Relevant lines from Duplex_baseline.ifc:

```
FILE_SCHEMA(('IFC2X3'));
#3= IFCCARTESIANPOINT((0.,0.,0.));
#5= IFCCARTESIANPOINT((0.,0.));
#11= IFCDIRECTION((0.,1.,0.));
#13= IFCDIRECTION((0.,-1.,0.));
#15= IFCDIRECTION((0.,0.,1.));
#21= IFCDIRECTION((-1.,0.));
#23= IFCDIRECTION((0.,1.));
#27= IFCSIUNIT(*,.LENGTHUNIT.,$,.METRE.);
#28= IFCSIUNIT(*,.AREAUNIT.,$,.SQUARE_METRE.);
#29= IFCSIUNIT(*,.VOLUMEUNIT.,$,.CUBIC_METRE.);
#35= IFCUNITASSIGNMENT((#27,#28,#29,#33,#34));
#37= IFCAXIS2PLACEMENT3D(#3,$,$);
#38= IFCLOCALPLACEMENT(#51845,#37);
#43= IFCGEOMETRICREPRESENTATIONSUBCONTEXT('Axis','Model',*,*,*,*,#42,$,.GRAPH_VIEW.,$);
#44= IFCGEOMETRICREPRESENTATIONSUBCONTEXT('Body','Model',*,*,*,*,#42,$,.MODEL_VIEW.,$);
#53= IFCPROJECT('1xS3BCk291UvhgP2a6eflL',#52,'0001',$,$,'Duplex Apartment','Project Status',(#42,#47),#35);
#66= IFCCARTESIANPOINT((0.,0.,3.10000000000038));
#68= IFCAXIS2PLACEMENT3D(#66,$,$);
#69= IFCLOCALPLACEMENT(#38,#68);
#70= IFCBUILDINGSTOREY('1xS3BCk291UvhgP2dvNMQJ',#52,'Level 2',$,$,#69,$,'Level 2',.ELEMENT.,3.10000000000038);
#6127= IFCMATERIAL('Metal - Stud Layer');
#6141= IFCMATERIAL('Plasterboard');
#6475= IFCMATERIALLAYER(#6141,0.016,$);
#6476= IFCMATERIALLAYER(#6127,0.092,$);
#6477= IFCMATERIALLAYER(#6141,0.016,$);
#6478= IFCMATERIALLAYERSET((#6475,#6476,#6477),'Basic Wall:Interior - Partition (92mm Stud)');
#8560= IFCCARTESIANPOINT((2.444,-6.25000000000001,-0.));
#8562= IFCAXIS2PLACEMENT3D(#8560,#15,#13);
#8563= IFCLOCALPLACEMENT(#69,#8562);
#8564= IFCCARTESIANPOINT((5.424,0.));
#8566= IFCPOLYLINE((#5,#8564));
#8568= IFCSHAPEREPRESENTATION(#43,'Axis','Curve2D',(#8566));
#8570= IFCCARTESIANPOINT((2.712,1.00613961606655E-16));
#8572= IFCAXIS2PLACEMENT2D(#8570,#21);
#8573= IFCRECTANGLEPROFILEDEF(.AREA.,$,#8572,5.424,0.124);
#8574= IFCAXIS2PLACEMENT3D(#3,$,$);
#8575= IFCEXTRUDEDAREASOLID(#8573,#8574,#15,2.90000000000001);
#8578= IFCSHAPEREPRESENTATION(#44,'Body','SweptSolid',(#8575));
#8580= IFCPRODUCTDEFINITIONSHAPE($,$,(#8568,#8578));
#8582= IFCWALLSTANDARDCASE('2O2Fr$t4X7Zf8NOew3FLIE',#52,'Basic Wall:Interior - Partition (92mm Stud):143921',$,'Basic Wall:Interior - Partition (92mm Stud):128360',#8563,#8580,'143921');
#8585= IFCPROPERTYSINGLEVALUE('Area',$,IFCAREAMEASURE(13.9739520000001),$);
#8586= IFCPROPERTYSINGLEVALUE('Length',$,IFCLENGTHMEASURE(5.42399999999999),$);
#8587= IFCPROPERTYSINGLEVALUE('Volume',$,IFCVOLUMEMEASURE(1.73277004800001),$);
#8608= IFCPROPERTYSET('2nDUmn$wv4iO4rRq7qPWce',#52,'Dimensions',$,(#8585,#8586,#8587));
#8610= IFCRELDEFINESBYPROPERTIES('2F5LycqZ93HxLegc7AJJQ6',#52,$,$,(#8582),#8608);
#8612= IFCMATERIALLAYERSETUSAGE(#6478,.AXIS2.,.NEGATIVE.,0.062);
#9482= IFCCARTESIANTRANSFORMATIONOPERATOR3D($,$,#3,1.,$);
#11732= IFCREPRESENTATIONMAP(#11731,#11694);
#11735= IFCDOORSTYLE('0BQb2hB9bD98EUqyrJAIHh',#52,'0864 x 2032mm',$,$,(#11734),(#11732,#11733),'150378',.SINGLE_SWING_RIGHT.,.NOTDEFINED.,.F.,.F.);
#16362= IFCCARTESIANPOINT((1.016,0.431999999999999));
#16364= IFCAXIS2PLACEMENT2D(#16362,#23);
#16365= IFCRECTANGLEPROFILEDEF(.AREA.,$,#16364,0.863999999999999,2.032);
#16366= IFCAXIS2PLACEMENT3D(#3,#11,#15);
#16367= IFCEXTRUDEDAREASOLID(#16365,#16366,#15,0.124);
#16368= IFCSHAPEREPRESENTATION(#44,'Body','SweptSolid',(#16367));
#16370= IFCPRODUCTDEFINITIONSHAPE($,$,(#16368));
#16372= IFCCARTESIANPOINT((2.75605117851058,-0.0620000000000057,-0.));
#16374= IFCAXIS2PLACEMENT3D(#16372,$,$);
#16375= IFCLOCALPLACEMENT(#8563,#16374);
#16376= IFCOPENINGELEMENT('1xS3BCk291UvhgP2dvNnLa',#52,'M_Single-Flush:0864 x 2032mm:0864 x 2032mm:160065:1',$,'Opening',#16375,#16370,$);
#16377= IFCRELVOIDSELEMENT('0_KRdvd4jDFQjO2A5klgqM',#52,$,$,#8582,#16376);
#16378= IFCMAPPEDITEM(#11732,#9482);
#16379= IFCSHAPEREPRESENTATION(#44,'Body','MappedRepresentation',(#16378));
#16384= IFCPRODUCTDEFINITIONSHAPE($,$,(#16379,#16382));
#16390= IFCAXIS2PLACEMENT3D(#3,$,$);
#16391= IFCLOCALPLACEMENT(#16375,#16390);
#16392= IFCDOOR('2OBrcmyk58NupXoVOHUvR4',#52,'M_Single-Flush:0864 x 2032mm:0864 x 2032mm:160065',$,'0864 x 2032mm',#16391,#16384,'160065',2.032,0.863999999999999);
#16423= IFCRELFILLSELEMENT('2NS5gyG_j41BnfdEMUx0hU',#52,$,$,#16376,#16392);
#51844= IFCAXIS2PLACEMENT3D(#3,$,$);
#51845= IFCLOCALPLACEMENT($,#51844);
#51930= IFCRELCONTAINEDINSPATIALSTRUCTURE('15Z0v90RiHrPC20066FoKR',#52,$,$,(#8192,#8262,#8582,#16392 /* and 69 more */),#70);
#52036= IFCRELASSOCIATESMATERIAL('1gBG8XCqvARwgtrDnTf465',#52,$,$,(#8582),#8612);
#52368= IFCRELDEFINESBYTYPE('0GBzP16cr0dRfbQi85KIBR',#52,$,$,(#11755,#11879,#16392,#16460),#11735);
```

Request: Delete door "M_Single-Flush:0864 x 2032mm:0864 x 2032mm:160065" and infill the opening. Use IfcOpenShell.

```python
import ifcopenshell
import ifcopenshell.api.feature
import ifcopenshell.api.pset
import ifcopenshell.api.root
import ifcopenshell.geom
import ifcopenshell.util.element
import ifcopenshell.util.shape
import ifcopenshell.util.unit

model = ifcopenshell.open("Duplex_baseline.ifc")
area_scale = ifcopenshell.util.unit.calculate_unit_scale(model, "AREAUNIT")
volume_scale = ifcopenshell.util.unit.calculate_unit_scale(model, "VOLUMEUNIT")
settings = ifcopenshell.geom.settings()


def volume(element):
    """Net volume in cubic metres, openings subtracted."""
    shape = ifcopenshell.geom.create_shape(settings, element)
    return ifcopenshell.util.shape.get_volume(shape.geometry)


door = model.by_guid("2OBrcmyk58NupXoVOHUvR4")
opening = door.FillsVoids[0].RelatingOpeningElement
wall = opening.VoidsElements[0].RelatingBuildingElement
before = volume(wall)

ifcopenshell.api.root.remove_product(model, product=door)
ifcopenshell.api.feature.remove_feature(model, feature=opening)

after = volume(wall)
thickness = 0.124  # wall thickness in metres

# Update the wall's stored quantities.
pset = model.by_id(ifcopenshell.util.element.get_pset(wall, "Dimensions", should_inherit=False)["id"])
ifcopenshell.api.pset.edit_pset(model, pset=pset, properties={
    "Area": model.create_entity("IfcAreaMeasure", after / thickness / area_scale),
    "Volume": model.create_entity("IfcVolumeMeasure", after / volume_scale),
})

print(f"wall volume {before:.3f} -> {after:.3f} m3")

model.write("Duplex_baseline_edited.ifc")
```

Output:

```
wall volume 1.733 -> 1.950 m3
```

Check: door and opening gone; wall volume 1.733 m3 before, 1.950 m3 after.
